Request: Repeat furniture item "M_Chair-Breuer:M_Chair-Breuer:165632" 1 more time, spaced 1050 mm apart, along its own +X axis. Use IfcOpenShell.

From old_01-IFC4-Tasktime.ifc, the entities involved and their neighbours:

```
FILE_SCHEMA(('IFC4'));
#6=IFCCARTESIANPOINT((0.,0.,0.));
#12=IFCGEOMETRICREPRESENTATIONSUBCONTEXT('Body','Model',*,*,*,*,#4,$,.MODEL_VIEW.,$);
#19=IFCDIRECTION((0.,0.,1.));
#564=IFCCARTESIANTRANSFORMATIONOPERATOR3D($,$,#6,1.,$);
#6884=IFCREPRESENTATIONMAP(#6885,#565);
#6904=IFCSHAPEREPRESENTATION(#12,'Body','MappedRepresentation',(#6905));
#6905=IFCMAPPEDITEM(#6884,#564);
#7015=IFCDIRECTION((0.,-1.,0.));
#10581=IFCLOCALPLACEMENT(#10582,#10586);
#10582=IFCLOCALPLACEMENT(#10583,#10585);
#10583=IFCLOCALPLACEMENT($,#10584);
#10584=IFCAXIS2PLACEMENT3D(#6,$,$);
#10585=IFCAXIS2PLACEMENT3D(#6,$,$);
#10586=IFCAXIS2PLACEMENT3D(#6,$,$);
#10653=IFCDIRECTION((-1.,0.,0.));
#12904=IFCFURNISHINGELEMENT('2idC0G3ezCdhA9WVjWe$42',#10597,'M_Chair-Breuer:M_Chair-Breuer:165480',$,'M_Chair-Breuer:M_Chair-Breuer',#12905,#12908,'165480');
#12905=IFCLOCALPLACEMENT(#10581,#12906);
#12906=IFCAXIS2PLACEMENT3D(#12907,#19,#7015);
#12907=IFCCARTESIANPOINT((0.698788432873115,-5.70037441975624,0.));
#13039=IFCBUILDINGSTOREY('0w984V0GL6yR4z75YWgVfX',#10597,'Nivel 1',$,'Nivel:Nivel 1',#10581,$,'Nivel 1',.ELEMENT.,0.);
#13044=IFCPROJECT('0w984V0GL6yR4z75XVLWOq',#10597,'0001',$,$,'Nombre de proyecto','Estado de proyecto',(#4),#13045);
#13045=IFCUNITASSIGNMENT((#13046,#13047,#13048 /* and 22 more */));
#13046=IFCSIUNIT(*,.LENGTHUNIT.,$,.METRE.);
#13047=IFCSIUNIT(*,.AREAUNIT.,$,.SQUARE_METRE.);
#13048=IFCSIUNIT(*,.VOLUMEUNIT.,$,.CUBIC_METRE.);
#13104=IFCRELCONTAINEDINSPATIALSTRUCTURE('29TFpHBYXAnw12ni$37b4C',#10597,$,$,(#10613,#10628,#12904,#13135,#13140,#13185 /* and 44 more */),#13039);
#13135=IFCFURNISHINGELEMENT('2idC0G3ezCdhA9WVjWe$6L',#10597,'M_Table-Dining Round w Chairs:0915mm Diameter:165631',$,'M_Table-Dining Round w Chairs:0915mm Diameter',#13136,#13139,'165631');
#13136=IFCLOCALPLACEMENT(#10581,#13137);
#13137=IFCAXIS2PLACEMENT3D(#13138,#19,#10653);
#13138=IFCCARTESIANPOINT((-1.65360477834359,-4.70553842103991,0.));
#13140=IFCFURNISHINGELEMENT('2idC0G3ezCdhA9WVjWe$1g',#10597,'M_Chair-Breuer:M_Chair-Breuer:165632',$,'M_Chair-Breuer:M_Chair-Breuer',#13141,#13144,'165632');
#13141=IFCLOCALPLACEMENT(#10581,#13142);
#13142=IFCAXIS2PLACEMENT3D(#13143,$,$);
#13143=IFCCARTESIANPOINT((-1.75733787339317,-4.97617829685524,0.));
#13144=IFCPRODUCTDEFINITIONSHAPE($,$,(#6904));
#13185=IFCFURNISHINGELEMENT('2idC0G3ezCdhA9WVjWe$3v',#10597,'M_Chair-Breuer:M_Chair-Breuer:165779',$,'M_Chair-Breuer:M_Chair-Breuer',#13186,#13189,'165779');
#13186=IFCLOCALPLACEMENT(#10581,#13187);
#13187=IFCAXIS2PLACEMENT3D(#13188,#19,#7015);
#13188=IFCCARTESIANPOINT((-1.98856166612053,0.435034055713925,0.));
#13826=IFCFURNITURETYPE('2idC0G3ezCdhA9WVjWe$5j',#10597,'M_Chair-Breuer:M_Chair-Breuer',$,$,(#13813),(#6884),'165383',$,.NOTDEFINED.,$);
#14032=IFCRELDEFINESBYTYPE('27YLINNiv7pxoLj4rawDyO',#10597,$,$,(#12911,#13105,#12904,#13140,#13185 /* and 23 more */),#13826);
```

```python
import ifcopenshell
import ifcopenshell.api.geometry
import ifcopenshell.api.root
import ifcopenshell.util.element
import ifcopenshell.util.placement
import ifcopenshell.util.unit

model = ifcopenshell.open("old_01-IFC4-Tasktime.ifc")
unit_scale = ifcopenshell.util.unit.calculate_unit_scale(model)


def reuse_history(source, copy):
    """copy_class also copies each property set's owner history, people and application; keep the originals."""
    for rel in copy.IsDefinedBy:
        if rel.is_a("IfcRelDefinesByProperties") and (history := rel.RelatingPropertyDefinition.OwnerHistory):
            rel.RelatingPropertyDefinition.OwnerHistory = source.OwnerHistory
            ifcopenshell.util.element.remove_deep2(model, history)


source = model.by_guid("2idC0G3ezCdhA9WVjWe$1g")
base = ifcopenshell.util.placement.get_local_placement(source.ObjectPlacement)
step = base[:3, 0] * 1.05 / unit_scale

for i in range(1, 2):
    copy = ifcopenshell.api.root.copy_class(model, product=source)
    copy.Representation = ifcopenshell.util.element.copy_deep(
        model, source.Representation, exclude=["IfcGeometricRepresentationContext", "IfcRepresentationMap"]
    )
    copy.Name = "M_Chair-Breuer:M_Chair-Breuer"
    copy.Tag = None
    reuse_history(source, copy)
    matrix = base.copy()
    matrix[:3, 3] += i * step
    print("added at", matrix[:3, 3].round(3) + 0.0)
    ifcopenshell.api.geometry.edit_object_placement(model, product=copy, matrix=matrix, is_si=False)

model.write("old_01-IFC4-Tasktime_rev.ifc")
```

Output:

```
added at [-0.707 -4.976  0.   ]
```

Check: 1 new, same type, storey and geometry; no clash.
